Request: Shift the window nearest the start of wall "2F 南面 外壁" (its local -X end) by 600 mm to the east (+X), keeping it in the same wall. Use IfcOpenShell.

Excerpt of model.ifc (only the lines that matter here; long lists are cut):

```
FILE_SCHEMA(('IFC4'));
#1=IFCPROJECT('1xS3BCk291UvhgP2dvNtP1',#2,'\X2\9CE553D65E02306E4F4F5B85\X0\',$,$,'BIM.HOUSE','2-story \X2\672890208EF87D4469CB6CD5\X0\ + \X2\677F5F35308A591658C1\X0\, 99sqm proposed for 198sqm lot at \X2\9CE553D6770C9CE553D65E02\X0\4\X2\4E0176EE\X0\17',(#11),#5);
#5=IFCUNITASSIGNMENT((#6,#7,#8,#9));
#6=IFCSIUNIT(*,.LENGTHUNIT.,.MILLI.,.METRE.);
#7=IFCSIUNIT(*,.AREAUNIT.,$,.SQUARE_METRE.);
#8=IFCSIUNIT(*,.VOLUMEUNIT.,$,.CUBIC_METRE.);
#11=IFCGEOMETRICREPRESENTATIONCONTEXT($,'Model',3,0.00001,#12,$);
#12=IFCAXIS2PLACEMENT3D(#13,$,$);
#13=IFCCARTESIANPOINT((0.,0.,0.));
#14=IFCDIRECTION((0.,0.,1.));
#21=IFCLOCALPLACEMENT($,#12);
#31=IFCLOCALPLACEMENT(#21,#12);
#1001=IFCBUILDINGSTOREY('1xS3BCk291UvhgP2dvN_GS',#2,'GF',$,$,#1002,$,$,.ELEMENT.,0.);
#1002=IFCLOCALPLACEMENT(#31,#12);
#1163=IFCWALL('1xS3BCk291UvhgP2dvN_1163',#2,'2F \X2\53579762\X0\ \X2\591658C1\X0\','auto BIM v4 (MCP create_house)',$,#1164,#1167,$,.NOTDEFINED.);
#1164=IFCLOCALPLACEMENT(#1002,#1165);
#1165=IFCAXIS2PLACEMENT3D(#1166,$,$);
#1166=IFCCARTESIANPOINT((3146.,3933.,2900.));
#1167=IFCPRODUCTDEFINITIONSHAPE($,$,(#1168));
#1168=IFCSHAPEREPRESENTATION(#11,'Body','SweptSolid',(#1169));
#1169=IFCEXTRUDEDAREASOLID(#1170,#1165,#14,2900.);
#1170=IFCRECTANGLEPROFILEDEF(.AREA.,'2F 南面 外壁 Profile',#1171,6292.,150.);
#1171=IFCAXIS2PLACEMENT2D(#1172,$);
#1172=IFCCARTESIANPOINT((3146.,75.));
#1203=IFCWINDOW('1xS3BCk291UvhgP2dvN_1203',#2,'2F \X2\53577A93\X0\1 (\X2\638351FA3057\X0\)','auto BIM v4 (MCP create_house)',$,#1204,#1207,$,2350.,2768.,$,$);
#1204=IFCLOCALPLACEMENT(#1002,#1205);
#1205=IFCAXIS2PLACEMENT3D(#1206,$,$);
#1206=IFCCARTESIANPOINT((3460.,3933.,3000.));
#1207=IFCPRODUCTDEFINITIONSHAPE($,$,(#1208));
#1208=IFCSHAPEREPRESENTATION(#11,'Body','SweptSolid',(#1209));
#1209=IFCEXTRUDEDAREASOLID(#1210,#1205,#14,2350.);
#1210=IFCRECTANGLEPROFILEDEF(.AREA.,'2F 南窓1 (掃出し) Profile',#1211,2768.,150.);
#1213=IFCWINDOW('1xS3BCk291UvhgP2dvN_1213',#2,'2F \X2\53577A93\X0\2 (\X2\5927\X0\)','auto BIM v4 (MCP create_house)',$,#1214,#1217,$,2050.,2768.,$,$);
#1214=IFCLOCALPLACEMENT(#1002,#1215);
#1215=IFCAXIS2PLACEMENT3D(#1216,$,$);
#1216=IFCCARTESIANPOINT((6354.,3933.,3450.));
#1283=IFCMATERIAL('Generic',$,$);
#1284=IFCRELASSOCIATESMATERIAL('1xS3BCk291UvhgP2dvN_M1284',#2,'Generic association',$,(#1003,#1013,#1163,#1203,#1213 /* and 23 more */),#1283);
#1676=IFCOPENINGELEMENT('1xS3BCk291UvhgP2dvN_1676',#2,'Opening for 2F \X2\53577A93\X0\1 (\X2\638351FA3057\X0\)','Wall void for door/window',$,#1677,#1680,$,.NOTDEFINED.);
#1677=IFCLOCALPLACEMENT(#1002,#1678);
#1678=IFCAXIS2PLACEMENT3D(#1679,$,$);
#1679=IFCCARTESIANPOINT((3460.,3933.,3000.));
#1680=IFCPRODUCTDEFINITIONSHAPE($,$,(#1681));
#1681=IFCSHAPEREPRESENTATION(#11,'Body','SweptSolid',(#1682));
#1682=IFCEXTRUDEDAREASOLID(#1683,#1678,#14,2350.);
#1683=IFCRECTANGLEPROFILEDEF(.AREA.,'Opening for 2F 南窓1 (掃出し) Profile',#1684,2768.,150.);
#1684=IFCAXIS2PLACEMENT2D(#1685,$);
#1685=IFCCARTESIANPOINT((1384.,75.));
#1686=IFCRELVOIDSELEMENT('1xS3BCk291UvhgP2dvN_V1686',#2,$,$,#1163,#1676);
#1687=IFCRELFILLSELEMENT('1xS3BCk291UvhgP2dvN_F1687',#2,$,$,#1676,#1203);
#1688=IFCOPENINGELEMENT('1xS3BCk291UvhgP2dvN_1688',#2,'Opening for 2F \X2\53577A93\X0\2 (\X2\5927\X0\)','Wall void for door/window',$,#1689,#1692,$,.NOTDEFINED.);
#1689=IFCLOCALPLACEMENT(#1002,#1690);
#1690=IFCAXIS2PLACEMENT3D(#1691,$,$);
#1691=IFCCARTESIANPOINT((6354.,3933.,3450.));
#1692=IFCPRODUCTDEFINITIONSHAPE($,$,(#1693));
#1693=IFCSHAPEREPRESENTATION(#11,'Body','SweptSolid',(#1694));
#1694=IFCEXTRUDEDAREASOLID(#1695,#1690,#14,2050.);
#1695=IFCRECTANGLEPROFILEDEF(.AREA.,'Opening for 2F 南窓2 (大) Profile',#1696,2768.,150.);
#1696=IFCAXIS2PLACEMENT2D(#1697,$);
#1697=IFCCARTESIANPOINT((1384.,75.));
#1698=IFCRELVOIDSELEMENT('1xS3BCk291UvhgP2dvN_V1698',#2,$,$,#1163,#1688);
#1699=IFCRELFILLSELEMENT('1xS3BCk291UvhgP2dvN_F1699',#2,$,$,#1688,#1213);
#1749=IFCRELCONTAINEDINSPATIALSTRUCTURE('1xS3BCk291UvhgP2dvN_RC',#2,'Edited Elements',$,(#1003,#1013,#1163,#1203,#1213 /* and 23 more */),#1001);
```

```python
import ifcopenshell
import ifcopenshell.api.geometry
import ifcopenshell.util.placement

model = ifcopenshell.open("model.ifc")

window = model.by_id(1203)
opening = window.FillsVoids[0].RelatingOpeningElement
wall = opening.VoidsElements[0].RelatingBuildingElement

wall_matrix = ifcopenshell.util.placement.get_local_placement(wall.ObjectPlacement)
shift = wall_matrix[:3, 0] * 600.0
before = ifcopenshell.util.placement.get_local_placement(window.ObjectPlacement)[:3, 3].copy()

# The window is not placed relative to its opening, so move both.
for product in (opening, window):
    matrix = ifcopenshell.util.placement.get_local_placement(product.ObjectPlacement)
    matrix[:3, 3] += shift
    ifcopenshell.api.geometry.edit_object_placement(model, product=product, matrix=matrix, is_si=False)

after = ifcopenshell.util.placement.get_local_placement(window.ObjectPlacement)[:3, 3]
print("window moved by", (after - before).round(3) + 0.0)

model.write("model_edited.ifc")
```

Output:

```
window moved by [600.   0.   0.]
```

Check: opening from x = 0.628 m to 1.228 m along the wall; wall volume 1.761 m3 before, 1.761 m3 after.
